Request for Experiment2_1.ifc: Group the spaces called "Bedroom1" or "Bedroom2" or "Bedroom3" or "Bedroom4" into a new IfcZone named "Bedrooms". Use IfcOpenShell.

First a look at what the model holds.

```python
import ifcopenshell

model = ifcopenshell.open("Experiment2_1.ifc")
print(model.schema)
seen = {}
for space in model.by_type("IfcSpace"):
    seen[space.LongName] = seen.get(space.LongName, 0) + 1
for name, count in sorted(seen.items(), key=str):
    print(count, "x", name)
print("zones:", [z.Name for z in model.by_type("IfcZone")][:20])
```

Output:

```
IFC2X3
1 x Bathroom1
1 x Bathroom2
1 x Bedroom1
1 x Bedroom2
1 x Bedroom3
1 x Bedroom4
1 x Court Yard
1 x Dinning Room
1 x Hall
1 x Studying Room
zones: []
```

```python
import ifcopenshell
import ifcopenshell.api.group
import ifcopenshell.api.root

model = ifcopenshell.open("Experiment2_1.ifc")

names = {"Bedroom1", "Bedroom2", "Bedroom3", "Bedroom4"}
spaces = [s for s in model.by_type("IfcSpace") if s.LongName in names]

zone = ifcopenshell.api.root.create_entity(model, ifc_class="IfcZone", name="Bedrooms")
ifcopenshell.api.group.assign_group(model, products=spaces, group=zone)
print(len(spaces), "spaces in", zone.Name)

model.write("Experiment2_1_v2.ifc")
```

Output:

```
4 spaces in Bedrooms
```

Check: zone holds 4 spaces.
